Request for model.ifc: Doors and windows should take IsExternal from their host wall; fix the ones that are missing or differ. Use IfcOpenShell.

First a look at what the model holds.

```python
import ifcopenshell
import ifcopenshell.util.element

model = ifcopenshell.open("model.ifc")
print(model.schema)
seen = {}
for e in model.by_type("IfcDoor") + model.by_type("IfcWindow"):
    if not e.FillsVoids:
        continue
    host = e.FillsVoids[0].RelatingOpeningElement.VoidsElements[0].RelatingBuildingElement
    own = ifcopenshell.util.element.get_pset(e, f"Pset_{e.is_a()[3:].removesuffix('StandardCase')}Common", "IsExternal")
    wall = ifcopenshell.util.element.get_pset(host, "Pset_WallCommon", "IsExternal")
    seen[e.is_a(), own, wall] = seen.get((e.is_a(), own, wall), 0) + 1
for (cls, own, wall), count in sorted(seen.items(), key=str):
    print(count, cls, "IsExternal:", own, "| host wall:", wall)
```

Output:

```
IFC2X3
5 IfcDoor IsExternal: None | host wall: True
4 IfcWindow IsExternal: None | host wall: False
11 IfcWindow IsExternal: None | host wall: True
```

```python
import ifcopenshell
import ifcopenshell.api.pset
import ifcopenshell.util.element

model = ifcopenshell.open("model.ifc")

count = 0
for ifc_class, pset_name in (("IfcDoor", "Pset_DoorCommon"), ("IfcWindow", "Pset_WindowCommon")):
    for e in model.by_type(ifc_class):
        if not e.FillsVoids:
            continue
        host = e.FillsVoids[0].RelatingOpeningElement.VoidsElements[0].RelatingBuildingElement
        external = ifcopenshell.util.element.get_pset(host, "Pset_WallCommon", "IsExternal")
        if external is None or ifcopenshell.util.element.get_pset(e, pset_name, "IsExternal") == external:
            continue
        pset = ifcopenshell.api.pset.add_pset(model, product=e, name=pset_name)
        ifcopenshell.api.pset.edit_pset(model, pset=pset, properties={"IsExternal": external})
        count += 1

print(count, "updated")

model.write("model_rev.ifc")
```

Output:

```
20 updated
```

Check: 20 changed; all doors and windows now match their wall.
